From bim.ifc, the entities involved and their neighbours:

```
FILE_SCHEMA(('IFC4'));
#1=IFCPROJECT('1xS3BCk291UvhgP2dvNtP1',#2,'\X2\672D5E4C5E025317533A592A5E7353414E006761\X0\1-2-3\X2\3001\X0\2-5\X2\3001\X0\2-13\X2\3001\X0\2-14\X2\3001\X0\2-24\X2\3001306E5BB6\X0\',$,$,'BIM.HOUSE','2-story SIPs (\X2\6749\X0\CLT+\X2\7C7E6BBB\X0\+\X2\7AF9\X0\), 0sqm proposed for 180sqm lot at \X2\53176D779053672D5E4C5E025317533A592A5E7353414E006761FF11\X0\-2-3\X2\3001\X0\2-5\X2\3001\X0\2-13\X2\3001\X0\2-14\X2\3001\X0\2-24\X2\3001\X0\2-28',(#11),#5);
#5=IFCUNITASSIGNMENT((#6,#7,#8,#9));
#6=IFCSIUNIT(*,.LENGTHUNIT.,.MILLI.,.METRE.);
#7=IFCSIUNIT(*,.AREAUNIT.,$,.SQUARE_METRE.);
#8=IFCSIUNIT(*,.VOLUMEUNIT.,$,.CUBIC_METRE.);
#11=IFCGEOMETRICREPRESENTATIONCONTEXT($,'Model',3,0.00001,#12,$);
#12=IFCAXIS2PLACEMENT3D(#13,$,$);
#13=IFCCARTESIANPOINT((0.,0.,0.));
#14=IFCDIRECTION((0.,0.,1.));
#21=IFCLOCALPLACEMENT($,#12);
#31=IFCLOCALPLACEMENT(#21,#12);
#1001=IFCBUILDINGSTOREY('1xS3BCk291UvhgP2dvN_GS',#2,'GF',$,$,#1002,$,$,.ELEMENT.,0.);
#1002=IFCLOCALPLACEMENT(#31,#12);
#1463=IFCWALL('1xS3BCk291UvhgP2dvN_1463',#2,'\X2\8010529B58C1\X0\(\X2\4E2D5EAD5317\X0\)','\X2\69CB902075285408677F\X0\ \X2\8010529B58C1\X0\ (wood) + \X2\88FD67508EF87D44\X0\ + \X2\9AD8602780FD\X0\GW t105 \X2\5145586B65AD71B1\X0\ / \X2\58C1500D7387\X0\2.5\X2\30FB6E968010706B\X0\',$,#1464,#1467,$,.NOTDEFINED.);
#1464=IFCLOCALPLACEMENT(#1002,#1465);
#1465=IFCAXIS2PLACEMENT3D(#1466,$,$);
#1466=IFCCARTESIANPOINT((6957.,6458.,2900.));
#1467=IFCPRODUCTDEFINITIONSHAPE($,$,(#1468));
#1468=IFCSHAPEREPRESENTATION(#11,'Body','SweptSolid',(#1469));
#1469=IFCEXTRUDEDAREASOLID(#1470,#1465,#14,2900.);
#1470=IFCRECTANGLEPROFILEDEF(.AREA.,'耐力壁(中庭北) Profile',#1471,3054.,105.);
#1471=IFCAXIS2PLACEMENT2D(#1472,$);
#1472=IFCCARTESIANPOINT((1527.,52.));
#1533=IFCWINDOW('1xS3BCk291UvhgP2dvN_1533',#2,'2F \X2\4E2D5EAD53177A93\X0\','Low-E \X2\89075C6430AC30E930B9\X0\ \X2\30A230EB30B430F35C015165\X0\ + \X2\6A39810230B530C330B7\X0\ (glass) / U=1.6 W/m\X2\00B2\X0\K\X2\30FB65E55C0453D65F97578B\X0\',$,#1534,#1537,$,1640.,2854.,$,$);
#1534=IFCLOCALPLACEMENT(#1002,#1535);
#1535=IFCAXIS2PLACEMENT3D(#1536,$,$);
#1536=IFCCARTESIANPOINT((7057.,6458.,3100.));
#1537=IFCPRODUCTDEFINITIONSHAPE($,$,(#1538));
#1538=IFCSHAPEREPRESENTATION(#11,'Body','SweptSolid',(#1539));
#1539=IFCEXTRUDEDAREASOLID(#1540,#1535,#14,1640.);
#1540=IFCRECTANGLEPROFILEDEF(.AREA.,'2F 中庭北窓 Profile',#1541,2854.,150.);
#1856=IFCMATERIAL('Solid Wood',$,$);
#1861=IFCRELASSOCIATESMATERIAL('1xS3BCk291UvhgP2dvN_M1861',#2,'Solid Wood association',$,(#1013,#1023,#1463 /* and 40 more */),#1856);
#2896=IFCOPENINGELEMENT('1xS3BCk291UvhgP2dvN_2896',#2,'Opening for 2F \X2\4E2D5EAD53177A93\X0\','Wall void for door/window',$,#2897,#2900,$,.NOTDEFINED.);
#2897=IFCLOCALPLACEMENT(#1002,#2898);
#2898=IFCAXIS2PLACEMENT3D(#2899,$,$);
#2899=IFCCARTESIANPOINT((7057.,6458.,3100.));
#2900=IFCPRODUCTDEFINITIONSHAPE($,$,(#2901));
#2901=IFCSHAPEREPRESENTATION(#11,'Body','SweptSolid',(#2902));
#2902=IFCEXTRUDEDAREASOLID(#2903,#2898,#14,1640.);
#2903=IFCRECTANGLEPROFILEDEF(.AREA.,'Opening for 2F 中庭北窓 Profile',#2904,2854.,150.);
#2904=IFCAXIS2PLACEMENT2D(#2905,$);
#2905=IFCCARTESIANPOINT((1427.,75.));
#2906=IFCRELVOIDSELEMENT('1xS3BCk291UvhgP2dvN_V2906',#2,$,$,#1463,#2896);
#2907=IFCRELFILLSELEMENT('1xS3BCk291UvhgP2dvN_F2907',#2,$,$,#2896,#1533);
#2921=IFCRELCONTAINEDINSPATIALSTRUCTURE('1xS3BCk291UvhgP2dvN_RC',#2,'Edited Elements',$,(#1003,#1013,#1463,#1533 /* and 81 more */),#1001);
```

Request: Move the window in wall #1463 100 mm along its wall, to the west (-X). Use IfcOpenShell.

```python
import ifcopenshell
import ifcopenshell.api.geometry
import ifcopenshell.util.placement

model = ifcopenshell.open("bim.ifc")

window = model.by_id(1533)
opening = window.FillsVoids[0].RelatingOpeningElement
wall = opening.VoidsElements[0].RelatingBuildingElement

wall_matrix = ifcopenshell.util.placement.get_local_placement(wall.ObjectPlacement)
shift = wall_matrix[:3, 0] * -100.0
before = ifcopenshell.util.placement.get_local_placement(window.ObjectPlacement)[:3, 3].copy()

# The window is not placed relative to its opening, so move both.
for product in (opening, window):
    matrix = ifcopenshell.util.placement.get_local_placement(product.ObjectPlacement)
    matrix[:3, 3] += shift
    ifcopenshell.api.geometry.edit_object_placement(model, product=product, matrix=matrix, is_si=False)

after = ifcopenshell.util.placement.get_local_placement(window.ObjectPlacement)[:3, 3]
print("window moved by", (after - before).round(3) + 0.0)

model.write("bim_edited.ifc")
```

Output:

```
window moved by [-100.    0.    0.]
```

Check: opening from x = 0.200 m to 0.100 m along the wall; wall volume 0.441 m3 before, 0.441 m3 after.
